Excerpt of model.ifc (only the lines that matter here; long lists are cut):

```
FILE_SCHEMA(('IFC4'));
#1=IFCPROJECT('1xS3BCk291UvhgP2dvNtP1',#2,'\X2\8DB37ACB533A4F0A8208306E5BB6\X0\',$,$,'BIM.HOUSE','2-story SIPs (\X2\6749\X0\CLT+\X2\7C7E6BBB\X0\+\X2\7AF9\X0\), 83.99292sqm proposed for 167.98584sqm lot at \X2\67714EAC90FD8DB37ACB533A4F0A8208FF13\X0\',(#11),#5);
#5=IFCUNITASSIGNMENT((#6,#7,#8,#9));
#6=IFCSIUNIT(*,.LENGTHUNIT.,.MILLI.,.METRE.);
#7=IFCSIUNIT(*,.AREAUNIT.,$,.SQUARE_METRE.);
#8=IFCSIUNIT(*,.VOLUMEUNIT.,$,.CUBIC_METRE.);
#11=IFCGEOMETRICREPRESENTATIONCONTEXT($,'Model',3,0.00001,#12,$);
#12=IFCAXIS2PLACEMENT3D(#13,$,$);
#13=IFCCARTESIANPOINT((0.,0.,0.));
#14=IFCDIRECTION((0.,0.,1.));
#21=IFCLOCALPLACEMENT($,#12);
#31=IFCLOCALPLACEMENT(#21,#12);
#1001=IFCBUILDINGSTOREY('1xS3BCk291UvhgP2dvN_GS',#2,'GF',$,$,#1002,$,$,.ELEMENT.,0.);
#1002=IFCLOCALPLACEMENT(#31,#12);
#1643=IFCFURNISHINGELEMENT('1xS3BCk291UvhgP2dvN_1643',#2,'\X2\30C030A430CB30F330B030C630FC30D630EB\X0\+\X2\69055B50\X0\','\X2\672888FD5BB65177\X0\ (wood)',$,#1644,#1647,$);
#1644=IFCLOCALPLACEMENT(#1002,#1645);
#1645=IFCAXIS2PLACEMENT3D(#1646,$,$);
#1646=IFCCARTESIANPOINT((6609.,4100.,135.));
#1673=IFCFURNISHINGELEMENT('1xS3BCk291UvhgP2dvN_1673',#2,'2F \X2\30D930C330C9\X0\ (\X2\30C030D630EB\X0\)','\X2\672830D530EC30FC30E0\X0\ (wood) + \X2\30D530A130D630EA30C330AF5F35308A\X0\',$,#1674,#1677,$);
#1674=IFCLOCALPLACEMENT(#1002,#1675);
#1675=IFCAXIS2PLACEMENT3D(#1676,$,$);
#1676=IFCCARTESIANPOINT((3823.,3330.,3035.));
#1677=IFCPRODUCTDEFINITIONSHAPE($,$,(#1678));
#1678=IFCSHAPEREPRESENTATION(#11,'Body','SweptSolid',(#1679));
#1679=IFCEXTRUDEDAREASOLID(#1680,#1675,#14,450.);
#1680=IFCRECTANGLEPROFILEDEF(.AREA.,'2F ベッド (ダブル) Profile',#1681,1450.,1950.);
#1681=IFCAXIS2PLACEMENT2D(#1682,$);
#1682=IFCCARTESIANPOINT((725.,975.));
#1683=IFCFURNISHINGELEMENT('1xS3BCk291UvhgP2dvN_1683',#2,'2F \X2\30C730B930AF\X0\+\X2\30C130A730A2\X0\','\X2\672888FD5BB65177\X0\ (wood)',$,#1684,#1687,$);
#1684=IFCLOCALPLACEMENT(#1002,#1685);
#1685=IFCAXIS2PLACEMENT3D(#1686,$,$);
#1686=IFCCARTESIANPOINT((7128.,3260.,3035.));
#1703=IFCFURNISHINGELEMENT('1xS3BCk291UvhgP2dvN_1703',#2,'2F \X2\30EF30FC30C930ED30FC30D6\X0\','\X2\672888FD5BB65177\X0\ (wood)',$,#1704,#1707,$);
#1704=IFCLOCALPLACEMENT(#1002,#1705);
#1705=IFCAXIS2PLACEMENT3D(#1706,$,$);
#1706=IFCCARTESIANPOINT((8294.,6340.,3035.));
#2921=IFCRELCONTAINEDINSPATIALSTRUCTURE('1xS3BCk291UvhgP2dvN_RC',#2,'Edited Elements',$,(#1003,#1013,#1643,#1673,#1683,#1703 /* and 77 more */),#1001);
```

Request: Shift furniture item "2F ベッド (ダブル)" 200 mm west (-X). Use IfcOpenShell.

```python
import ifcopenshell
import ifcopenshell.api.geometry
import ifcopenshell.util.placement

model = ifcopenshell.open("model.ifc")

item = model.by_id(1673)
matrix = ifcopenshell.util.placement.get_local_placement(item.ObjectPlacement)
matrix[0, 3] -= 200.0
ifcopenshell.api.geometry.edit_object_placement(model, product=item, matrix=matrix, is_si=False)

print(ifcopenshell.util.placement.get_local_placement(item.ObjectPlacement).round(3) + 0.0)

model.write("model_v2.ifc")
```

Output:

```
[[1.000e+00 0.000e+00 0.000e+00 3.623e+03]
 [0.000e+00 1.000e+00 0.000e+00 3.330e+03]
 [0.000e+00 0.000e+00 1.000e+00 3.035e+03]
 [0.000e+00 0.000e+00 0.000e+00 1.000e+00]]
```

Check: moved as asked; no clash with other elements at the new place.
